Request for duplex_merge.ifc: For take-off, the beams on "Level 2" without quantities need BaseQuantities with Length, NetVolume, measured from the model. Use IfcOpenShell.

First a look at what the model holds.

```python
import ifcopenshell
import ifcopenshell.util.element
import ifcopenshell.util.unit

model = ifcopenshell.open("duplex_merge.ifc")
print(model.schema)
for unit_type in ("LENGTHUNIT", "AREAUNIT", "VOLUMEUNIT"):
    print(unit_type, ifcopenshell.util.unit.calculate_unit_scale(model, unit_type))
storey = next(s for s in model.by_type("IfcBuildingStorey") if s.Name == "Level 2")
beams = [e for e in ifcopenshell.util.element.get_decomposition(storey) if e.is_a("IfcBeam")]
for e in sorted(beams, key=lambda e: e.id()):
    print(e.id(), e.is_a(), e.Name, list(ifcopenshell.util.element.get_psets(e, qtos_only=True)), sep=" | ")
```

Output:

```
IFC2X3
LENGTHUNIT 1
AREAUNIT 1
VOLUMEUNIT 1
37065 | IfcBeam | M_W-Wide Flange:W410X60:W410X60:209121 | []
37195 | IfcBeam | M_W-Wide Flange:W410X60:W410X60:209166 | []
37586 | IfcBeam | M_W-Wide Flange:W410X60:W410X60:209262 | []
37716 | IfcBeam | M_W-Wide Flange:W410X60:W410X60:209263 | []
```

```python
import ifcopenshell
import ifcopenshell.api.pset
import ifcopenshell.geom
import ifcopenshell.util.element
import ifcopenshell.util.shape
import ifcopenshell.util.unit

model = ifcopenshell.open("duplex_merge.ifc")
unit_scale = ifcopenshell.util.unit.calculate_unit_scale(model)
volume_scale = ifcopenshell.util.unit.calculate_unit_scale(model, "VOLUMEUNIT")
settings = ifcopenshell.geom.settings()

storey = next(s for s in model.by_type("IfcBuildingStorey") if s.Name == "Level 2")
beams = [e for e in ifcopenshell.util.element.get_decomposition(storey) if e.is_a("IfcBeam")]

for e in sorted(beams, key=lambda e: e.id()):
    if ifcopenshell.util.element.get_psets(e, qtos_only=True, should_inherit=False):
        continue
    # Geometry comes back in metres, in the element's own axes.
    shape = ifcopenshell.geom.create_shape(settings, e)
    values = {
        "Length": ifcopenshell.util.shape.get_max_xyz(shape.geometry) / unit_scale,
        "NetVolume": ifcopenshell.util.shape.get_volume(shape.geometry) / volume_scale,
    }
    qto = ifcopenshell.api.pset.add_qto(model, product=e, name="BaseQuantities")
    ifcopenshell.api.pset.edit_qto(model, qto=qto, properties=values)
    print(e.id(), {k: round(v, 3) for k, v in values.items()})

model.write("duplex_merge_edited.ifc")
```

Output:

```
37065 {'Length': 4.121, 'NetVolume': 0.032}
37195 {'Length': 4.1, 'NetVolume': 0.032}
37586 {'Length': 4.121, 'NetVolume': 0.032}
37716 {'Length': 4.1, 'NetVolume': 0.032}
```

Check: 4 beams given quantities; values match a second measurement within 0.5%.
